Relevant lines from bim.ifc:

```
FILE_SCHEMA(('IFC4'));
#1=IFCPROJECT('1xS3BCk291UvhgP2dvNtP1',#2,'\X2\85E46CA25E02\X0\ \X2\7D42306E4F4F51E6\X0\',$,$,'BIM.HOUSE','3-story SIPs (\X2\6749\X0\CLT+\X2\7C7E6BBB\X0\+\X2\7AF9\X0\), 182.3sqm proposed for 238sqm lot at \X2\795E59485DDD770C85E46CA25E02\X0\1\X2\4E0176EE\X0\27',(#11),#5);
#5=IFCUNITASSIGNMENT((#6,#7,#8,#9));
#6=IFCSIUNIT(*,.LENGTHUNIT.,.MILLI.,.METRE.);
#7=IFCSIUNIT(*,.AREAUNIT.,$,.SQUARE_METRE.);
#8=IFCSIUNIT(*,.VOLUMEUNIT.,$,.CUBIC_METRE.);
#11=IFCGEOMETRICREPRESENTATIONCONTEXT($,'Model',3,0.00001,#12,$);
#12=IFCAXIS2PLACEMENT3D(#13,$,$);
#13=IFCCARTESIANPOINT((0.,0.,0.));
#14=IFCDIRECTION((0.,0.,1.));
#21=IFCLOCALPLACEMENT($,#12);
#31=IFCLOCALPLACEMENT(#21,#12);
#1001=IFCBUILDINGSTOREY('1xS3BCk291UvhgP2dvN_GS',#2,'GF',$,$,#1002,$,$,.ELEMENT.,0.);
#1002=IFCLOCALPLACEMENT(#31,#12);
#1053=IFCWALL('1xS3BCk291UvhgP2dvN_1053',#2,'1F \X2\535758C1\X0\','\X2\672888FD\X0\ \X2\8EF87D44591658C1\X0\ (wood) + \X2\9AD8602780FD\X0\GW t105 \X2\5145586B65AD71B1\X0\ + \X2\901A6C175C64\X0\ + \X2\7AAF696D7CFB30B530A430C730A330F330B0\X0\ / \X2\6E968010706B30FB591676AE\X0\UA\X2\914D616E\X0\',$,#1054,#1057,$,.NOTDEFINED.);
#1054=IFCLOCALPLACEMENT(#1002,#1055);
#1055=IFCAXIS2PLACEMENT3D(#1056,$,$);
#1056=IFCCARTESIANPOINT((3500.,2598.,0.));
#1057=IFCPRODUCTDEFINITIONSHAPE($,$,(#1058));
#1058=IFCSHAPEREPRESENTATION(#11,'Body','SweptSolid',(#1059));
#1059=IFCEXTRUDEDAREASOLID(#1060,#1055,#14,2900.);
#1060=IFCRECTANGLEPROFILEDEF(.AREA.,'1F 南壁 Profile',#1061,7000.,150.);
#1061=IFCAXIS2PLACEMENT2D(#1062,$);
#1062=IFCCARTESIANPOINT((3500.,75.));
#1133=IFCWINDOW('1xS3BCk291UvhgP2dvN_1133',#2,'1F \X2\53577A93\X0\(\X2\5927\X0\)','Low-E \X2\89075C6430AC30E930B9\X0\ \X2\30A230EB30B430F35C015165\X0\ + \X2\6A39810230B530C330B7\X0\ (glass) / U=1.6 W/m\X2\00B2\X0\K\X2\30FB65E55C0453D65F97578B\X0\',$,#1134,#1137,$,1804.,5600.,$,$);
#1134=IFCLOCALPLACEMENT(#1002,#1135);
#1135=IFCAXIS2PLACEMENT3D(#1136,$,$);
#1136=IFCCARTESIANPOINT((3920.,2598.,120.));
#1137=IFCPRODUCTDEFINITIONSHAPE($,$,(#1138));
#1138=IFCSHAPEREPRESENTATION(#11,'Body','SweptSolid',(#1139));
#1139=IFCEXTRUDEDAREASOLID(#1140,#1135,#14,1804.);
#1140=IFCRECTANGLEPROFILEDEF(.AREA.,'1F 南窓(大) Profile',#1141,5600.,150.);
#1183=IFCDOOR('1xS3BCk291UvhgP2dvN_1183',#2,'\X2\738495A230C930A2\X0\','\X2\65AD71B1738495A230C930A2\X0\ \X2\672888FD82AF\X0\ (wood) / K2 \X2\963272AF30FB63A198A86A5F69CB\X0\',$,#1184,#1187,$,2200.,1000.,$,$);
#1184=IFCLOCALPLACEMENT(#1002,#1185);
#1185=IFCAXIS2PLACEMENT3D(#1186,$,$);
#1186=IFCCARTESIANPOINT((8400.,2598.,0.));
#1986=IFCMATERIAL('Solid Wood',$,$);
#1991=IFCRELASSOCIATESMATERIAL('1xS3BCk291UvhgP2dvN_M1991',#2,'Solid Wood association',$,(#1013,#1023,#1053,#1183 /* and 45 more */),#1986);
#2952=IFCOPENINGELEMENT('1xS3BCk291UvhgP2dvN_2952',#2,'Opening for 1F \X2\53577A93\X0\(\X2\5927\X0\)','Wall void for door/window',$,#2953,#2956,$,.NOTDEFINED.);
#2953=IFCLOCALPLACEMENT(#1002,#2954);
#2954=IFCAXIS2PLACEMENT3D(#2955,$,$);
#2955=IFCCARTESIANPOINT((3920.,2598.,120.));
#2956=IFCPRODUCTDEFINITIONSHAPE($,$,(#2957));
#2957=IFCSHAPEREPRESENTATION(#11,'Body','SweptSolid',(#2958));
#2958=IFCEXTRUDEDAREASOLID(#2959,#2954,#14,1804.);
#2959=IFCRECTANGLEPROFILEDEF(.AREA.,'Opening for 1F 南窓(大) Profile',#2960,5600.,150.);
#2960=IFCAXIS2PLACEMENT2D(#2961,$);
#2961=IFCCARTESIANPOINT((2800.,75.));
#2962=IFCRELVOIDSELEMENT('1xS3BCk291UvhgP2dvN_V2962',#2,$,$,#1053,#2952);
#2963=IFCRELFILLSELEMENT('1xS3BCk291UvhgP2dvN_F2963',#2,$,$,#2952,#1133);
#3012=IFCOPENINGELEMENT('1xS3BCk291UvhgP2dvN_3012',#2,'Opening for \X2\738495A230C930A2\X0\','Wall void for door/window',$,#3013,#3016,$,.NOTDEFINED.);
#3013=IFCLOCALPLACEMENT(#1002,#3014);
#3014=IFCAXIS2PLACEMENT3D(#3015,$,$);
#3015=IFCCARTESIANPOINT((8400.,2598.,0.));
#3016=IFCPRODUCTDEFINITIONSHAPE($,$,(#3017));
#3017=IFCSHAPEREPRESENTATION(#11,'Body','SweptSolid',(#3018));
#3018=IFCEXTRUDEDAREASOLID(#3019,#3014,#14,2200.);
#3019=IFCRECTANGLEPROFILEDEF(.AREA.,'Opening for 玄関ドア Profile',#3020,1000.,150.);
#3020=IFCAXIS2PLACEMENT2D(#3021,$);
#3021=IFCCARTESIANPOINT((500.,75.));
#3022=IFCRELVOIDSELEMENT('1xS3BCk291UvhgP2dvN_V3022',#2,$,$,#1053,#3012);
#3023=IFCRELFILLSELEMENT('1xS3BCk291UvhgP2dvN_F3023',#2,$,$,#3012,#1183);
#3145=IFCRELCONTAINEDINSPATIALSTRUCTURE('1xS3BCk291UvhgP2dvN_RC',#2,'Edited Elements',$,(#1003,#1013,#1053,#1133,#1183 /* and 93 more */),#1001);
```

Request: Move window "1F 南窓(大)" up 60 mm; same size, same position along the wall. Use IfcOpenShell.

```python
import numpy as np
import ifcopenshell
import ifcopenshell.api.geometry
import ifcopenshell.util.placement
import ifcopenshell.util.unit

model = ifcopenshell.open("bim.ifc")
unit_scale = ifcopenshell.util.unit.calculate_unit_scale(model)

window = model.by_guid("1xS3BCk291UvhgP2dvN_1133")
opening = window.FillsVoids[0].RelatingOpeningElement
dz = 0.06 / unit_scale

shift = np.array([0.0, 0.0, dz])
# The window is not placed relative to its opening, so move both.
for product in (opening, window):
    matrix = ifcopenshell.util.placement.get_local_placement(product.ObjectPlacement)
    matrix[:3, 3] += shift
    ifcopenshell.api.geometry.edit_object_placement(model, product=product, matrix=matrix, is_si=False)

print(f"moved by {dz * unit_scale:+.3f} m")

model.write("bim_v2.ifc")
```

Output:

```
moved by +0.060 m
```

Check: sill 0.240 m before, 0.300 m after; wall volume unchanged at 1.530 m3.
